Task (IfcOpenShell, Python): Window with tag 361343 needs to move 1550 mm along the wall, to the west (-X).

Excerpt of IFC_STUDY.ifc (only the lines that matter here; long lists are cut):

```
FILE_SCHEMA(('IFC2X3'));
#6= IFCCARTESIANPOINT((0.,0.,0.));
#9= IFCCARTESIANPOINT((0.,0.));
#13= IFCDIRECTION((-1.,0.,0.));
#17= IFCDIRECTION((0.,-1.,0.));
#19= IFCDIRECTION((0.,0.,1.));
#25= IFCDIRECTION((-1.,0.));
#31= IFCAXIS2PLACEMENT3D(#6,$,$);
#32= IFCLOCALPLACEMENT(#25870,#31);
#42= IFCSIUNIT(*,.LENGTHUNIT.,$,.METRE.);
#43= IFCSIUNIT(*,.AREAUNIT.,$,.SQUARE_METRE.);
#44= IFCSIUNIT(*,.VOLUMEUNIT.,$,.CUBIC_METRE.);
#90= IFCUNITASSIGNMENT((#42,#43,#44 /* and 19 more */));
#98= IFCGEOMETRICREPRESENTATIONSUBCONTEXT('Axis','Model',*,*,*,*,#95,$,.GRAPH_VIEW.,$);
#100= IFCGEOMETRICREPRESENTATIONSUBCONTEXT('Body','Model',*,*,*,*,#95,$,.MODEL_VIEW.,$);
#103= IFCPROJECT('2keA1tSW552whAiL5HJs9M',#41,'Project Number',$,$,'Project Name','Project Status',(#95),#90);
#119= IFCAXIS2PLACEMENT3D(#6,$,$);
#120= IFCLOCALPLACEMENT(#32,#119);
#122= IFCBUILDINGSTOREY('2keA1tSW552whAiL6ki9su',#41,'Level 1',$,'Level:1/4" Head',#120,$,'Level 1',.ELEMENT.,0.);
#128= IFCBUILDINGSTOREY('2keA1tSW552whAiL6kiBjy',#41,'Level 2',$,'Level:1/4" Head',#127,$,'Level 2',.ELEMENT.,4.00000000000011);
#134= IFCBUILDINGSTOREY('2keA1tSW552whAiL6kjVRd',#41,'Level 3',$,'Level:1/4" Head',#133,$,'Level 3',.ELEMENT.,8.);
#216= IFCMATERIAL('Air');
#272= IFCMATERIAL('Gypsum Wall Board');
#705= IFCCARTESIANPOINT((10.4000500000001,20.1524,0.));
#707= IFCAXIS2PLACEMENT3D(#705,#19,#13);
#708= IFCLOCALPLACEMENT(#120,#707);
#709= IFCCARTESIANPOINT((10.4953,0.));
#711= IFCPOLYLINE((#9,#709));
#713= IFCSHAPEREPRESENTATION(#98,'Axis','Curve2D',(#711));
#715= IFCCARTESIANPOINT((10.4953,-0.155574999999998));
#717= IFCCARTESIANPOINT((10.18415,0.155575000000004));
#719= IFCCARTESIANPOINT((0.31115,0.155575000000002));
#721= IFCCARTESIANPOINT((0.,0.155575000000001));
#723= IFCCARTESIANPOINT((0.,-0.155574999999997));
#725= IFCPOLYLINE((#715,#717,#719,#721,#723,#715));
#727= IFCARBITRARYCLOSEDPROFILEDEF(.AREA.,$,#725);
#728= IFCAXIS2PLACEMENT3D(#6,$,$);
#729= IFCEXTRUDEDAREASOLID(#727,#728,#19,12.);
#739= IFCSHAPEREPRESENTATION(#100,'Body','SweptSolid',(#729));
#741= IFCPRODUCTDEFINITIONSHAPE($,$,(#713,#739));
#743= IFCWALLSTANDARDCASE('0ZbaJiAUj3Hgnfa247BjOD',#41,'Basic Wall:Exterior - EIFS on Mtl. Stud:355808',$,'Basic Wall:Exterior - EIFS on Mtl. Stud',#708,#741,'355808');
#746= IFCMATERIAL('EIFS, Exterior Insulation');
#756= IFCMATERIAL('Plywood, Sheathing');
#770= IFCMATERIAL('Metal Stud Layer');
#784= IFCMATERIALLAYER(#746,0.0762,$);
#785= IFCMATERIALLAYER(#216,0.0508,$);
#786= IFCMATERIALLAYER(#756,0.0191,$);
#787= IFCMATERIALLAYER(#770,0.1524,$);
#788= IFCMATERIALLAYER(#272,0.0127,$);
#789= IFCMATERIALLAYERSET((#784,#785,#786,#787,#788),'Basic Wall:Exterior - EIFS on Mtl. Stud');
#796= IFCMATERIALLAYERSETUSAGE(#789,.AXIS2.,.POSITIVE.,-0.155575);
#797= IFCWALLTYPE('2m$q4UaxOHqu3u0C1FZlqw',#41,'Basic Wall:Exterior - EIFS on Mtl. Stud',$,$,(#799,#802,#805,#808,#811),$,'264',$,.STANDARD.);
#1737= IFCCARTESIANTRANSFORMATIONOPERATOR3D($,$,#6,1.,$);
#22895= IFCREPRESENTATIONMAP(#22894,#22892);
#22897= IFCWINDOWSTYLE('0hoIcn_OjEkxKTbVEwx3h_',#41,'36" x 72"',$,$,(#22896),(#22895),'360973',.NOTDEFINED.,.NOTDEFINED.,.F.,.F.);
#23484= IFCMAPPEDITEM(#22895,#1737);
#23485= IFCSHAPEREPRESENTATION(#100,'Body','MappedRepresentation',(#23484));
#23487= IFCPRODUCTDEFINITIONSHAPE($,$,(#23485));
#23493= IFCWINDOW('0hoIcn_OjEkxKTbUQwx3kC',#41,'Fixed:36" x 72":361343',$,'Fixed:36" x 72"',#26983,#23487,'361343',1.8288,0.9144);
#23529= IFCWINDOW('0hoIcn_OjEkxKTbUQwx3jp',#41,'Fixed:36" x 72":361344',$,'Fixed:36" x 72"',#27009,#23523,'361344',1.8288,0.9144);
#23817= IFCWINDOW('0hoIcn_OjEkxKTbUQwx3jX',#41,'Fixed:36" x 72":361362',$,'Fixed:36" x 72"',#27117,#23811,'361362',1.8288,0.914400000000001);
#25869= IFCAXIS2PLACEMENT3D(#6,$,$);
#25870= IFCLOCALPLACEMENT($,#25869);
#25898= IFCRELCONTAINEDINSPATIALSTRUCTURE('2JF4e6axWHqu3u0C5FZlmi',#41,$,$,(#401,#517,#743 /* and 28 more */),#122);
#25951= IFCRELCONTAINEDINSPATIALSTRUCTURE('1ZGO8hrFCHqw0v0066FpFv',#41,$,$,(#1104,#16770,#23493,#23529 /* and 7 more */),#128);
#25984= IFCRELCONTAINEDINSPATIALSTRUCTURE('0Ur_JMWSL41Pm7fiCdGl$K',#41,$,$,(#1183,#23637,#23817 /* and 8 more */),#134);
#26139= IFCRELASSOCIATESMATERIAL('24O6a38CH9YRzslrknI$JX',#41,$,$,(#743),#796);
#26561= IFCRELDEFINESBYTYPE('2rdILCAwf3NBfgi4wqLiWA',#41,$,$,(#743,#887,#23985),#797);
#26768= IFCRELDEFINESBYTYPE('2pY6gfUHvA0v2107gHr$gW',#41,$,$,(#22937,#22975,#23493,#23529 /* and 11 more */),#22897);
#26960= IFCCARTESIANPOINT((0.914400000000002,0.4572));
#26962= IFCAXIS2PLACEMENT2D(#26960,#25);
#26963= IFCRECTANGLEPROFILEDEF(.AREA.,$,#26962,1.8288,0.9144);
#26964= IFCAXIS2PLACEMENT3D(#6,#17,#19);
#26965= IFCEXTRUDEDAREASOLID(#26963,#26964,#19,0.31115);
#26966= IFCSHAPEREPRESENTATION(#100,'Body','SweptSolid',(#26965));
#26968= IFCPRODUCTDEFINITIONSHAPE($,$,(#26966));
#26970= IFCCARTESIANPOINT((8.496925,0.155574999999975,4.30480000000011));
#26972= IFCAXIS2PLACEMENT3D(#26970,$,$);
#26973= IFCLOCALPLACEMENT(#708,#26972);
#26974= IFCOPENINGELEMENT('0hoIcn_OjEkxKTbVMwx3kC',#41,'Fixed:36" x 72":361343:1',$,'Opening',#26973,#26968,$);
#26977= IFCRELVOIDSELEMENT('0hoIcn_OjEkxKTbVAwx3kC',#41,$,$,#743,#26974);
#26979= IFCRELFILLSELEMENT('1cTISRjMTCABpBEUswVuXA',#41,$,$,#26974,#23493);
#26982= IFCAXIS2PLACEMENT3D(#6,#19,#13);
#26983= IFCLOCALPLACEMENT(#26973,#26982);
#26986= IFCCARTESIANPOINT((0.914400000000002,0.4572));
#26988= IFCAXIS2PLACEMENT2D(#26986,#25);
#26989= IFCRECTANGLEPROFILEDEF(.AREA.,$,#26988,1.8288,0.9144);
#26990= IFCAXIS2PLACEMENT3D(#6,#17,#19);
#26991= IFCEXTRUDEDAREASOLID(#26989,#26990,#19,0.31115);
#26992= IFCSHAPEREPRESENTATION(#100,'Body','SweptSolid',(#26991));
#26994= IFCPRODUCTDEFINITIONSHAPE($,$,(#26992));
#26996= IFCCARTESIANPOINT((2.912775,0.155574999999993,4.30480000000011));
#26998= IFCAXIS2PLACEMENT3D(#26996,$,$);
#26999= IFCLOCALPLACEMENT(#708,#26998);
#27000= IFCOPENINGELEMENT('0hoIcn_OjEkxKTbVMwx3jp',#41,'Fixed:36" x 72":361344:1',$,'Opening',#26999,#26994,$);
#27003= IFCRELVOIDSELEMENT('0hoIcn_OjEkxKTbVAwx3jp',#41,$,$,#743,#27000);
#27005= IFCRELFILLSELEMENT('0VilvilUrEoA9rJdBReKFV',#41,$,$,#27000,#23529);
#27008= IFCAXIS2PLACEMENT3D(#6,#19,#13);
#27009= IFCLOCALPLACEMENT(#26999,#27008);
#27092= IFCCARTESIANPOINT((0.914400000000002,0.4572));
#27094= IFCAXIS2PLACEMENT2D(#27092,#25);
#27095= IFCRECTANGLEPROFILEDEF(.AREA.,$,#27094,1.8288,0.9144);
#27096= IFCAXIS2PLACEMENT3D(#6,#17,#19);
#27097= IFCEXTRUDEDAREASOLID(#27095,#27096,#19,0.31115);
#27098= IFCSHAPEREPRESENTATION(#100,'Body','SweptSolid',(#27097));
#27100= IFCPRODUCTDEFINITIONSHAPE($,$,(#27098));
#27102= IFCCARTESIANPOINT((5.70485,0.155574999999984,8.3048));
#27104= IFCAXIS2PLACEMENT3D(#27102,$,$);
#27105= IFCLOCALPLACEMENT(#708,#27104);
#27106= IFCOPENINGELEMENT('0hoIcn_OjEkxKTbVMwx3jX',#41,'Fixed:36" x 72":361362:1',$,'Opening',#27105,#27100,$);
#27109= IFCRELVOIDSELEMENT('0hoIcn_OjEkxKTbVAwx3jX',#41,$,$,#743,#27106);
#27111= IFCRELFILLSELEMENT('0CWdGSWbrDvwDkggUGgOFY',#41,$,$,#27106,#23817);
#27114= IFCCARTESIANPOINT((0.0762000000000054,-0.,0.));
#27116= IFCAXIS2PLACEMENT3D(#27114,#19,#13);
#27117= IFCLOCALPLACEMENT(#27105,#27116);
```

```python
import ifcopenshell
import ifcopenshell.api.geometry
import ifcopenshell.util.placement
import ifcopenshell.util.unit

model = ifcopenshell.open("IFC_STUDY.ifc")
unit_scale = ifcopenshell.util.unit.calculate_unit_scale(model)

window = model.by_id(23493)
opening = window.FillsVoids[0].RelatingOpeningElement
wall = opening.VoidsElements[0].RelatingBuildingElement

wall_matrix = ifcopenshell.util.placement.get_local_placement(wall.ObjectPlacement)
shift = wall_matrix[:3, 0] * 1.55 / unit_scale
before = ifcopenshell.util.placement.get_local_placement(window.ObjectPlacement)[:3, 3].copy()

# The window is placed relative to its opening, so it follows when the opening moves.
matrix = ifcopenshell.util.placement.get_local_placement(opening.ObjectPlacement)
matrix[:3, 3] += shift
ifcopenshell.api.geometry.edit_object_placement(
    model, product=opening, matrix=matrix, is_si=False, should_transform_children=True
)

after = ifcopenshell.util.placement.get_local_placement(window.ObjectPlacement)[:3, 3]
print("window moved by", (after - before).round(3) + 0.0)

model.write("IFC_STUDY_rev.ifc")
```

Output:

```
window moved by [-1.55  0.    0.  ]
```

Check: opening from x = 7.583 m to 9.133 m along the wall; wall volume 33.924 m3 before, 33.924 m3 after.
